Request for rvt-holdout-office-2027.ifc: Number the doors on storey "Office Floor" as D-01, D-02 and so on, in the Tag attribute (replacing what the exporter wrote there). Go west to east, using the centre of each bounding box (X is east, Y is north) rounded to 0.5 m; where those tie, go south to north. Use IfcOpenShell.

First a look at what the model holds.

```python
import ifcopenshell
import ifcopenshell.util.element
import ifcopenshell.util.placement

model = ifcopenshell.open("rvt-holdout-office-2027.ifc")
print(model.schema)
storey = next(s for s in model.by_type("IfcBuildingStorey") if s.Name == "Office Floor")
doors = [e for e in ifcopenshell.util.element.get_decomposition(storey) if e.is_a("IfcDoor")]
for e in sorted(doors, key=lambda e: e.id()):
    origin = ifcopenshell.util.placement.get_local_placement(e.ObjectPlacement)[:3, 3]
    print(e.id(), e.Tag, e.Name, origin.round(2) + 0.0, sep=" | ")
```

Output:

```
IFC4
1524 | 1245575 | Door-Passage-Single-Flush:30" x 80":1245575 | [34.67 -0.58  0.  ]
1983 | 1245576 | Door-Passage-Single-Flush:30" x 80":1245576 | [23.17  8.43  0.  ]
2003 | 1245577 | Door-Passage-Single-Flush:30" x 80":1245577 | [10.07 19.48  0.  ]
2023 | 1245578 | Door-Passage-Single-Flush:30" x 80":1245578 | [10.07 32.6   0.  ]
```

```python
import ifcopenshell
import ifcopenshell.geom
import ifcopenshell.util.element
import ifcopenshell.util.shape

model = ifcopenshell.open("rvt-holdout-office-2027.ifc")
settings = ifcopenshell.geom.settings()
settings.set("use-world-coords", True)


def centre(element):
    shape = ifcopenshell.geom.create_shape(settings, element)
    return ifcopenshell.util.shape.get_bbox_centroid(shape.geometry)


storey = next(s for s in model.by_type("IfcBuildingStorey") if s.Name == "Office Floor")
doors = [e for e in ifcopenshell.util.element.get_decomposition(storey) if e.is_a("IfcDoor")]

# Insertion points can sit at a corner or the storey origin, so sort by the geometry (in metres).
centres = {e: centre(e) for e in doors}
doors.sort(key=lambda e: (round(centres[e][0] / 0.5), centres[e][1]))

for i, e in enumerate(doors, start=1):
    number = f"D-{i:02d}"
    e.Tag = number
    print(e.id(), number)

model.write("rvt-holdout-office-2027_edited.ifc")
```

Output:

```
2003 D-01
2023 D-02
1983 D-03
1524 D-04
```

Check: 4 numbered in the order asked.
